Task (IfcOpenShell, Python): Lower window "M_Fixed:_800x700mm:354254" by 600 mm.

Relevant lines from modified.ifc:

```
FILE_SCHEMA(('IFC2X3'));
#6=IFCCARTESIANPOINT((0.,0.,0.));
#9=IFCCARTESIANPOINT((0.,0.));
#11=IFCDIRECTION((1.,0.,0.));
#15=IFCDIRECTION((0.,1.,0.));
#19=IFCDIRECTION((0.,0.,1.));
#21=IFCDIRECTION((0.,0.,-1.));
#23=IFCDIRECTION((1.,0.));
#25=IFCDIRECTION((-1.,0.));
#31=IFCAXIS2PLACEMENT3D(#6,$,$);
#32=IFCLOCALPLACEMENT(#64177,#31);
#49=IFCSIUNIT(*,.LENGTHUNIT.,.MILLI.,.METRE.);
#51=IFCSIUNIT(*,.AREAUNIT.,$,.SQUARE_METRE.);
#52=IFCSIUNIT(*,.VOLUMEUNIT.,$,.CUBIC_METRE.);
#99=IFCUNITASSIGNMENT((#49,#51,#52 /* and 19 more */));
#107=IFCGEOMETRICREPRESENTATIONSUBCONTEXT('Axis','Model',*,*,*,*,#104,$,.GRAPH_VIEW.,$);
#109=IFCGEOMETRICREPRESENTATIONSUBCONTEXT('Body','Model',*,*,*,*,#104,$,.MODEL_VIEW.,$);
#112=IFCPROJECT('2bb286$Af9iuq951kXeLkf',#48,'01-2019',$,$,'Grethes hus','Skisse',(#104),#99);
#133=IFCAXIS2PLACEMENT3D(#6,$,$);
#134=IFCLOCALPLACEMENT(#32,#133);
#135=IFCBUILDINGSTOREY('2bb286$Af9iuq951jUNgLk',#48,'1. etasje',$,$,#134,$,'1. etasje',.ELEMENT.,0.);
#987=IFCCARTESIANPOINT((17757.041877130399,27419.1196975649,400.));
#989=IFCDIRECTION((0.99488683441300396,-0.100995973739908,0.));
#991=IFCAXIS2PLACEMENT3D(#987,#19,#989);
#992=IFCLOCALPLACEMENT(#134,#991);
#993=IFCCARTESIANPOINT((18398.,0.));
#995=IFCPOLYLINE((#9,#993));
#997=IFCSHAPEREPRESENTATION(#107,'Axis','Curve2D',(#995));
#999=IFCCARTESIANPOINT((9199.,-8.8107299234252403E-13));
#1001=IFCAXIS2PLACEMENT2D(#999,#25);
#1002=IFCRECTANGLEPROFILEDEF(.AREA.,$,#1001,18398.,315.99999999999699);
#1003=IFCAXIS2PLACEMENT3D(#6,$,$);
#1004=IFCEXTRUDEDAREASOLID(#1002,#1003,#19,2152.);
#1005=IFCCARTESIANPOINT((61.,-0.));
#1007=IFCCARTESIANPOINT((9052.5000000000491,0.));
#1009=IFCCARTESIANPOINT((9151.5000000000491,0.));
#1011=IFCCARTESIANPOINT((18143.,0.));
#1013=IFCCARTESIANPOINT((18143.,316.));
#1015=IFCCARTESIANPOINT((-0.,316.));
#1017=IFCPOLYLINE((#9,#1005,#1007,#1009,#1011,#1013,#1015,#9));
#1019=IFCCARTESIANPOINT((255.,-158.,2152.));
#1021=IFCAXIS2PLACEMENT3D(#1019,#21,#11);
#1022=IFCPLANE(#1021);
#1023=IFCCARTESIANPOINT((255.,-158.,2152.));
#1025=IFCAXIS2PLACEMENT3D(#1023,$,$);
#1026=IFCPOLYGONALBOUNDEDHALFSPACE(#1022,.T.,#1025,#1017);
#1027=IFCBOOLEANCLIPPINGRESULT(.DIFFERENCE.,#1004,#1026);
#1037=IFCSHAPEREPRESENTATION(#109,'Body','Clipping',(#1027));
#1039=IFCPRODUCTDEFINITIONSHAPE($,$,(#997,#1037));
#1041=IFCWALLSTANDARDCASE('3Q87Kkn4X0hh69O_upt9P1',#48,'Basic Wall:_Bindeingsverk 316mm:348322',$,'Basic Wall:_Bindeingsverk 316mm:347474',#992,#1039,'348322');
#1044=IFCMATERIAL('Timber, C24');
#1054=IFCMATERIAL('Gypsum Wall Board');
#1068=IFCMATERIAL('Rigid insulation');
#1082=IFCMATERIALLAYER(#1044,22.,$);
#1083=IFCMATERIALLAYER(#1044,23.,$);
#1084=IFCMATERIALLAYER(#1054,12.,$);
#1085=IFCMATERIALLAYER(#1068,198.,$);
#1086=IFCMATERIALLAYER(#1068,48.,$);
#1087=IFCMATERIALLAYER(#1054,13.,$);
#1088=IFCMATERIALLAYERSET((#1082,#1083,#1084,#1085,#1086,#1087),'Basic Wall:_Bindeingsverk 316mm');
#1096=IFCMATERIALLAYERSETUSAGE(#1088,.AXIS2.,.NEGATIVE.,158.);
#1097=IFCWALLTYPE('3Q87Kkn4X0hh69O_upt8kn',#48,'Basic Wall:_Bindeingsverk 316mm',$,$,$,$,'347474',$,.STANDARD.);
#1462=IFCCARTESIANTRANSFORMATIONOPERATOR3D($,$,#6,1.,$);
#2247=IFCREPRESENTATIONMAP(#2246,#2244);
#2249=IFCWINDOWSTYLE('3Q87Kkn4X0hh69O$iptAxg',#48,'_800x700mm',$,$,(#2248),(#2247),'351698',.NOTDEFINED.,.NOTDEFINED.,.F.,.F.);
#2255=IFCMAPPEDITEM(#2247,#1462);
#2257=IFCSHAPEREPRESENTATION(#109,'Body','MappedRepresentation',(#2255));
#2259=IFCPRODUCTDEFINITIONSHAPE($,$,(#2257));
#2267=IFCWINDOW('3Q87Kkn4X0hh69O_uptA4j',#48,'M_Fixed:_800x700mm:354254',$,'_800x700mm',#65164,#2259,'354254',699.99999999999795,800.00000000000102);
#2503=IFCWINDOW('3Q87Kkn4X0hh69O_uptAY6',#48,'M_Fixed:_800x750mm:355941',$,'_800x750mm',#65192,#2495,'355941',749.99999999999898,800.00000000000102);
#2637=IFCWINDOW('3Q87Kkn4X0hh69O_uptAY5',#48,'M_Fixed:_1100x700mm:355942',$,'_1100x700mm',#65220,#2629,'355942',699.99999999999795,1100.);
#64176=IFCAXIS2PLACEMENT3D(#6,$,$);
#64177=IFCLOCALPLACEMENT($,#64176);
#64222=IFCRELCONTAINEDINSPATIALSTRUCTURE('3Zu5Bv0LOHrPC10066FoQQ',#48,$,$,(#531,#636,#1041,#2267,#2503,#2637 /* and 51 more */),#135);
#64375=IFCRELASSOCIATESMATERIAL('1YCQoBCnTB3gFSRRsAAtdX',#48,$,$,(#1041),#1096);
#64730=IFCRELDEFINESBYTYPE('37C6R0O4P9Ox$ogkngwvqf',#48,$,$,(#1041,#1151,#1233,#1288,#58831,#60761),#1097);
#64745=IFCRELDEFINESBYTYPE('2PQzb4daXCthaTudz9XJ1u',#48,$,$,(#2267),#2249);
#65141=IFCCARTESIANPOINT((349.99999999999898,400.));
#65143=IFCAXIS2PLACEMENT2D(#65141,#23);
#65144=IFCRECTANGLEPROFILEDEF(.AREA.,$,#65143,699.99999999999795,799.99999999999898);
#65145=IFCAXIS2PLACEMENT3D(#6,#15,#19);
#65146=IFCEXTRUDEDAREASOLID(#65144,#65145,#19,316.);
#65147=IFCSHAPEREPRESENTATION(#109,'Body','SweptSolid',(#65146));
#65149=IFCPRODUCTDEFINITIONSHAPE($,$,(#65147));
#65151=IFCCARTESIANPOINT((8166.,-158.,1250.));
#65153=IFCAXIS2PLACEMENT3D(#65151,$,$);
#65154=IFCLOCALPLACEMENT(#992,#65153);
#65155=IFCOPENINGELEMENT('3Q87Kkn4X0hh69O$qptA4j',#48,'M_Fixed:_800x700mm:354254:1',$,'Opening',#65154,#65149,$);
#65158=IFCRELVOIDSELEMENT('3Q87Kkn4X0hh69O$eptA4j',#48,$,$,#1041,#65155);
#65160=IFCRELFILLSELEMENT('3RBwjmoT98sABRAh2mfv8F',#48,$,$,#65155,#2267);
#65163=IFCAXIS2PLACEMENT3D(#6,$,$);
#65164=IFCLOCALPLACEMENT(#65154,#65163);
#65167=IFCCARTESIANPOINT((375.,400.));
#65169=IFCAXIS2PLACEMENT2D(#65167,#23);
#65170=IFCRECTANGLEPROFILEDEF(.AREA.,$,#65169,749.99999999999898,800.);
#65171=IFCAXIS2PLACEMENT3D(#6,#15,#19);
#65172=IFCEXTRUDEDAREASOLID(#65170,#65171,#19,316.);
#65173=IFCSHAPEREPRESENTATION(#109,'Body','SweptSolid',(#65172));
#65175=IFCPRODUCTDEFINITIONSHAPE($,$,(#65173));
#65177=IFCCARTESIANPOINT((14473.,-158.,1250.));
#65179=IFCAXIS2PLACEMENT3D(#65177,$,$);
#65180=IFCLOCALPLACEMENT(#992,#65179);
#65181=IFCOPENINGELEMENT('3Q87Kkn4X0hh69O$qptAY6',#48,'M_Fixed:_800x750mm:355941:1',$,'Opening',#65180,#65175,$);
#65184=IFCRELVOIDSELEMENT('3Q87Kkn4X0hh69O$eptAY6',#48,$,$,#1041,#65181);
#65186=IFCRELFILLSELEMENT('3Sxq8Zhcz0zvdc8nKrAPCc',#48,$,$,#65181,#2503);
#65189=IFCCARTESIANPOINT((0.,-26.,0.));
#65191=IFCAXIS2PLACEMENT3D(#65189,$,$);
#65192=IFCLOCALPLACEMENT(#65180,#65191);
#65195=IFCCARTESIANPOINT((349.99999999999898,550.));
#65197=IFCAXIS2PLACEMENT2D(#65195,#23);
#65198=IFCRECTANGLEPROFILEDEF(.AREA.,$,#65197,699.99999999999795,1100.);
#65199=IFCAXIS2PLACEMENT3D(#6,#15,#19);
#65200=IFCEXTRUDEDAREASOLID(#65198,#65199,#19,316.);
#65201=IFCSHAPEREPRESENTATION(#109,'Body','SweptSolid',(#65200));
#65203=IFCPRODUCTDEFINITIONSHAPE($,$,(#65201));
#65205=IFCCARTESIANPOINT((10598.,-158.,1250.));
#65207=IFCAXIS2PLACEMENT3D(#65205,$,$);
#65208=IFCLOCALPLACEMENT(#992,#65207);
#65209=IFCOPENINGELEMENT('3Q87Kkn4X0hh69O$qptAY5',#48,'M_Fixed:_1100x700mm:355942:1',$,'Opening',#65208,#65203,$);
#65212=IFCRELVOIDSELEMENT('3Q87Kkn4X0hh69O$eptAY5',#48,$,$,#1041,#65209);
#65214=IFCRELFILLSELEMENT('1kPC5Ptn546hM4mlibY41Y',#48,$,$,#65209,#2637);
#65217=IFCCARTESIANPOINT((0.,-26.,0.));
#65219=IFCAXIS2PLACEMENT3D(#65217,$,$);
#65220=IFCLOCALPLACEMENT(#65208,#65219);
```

```python
import numpy as np
import ifcopenshell
import ifcopenshell.api.geometry
import ifcopenshell.util.placement
import ifcopenshell.util.unit

model = ifcopenshell.open("modified.ifc")
unit_scale = ifcopenshell.util.unit.calculate_unit_scale(model)

window = model.by_guid("3Q87Kkn4X0hh69O_uptA4j")
opening = window.FillsVoids[0].RelatingOpeningElement
dz = -600.0

shift = np.array([0.0, 0.0, dz])
# The window is placed relative to its opening, so it follows when the opening moves.
matrix = ifcopenshell.util.placement.get_local_placement(opening.ObjectPlacement)
matrix[:3, 3] += shift
ifcopenshell.api.geometry.edit_object_placement(
    model, product=opening, matrix=matrix, is_si=False, should_transform_children=True
)

print(f"moved by {dz * unit_scale:+.3f} m")

model.write("modified_rev.ifc")
```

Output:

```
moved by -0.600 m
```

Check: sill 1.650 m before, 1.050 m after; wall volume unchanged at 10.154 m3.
